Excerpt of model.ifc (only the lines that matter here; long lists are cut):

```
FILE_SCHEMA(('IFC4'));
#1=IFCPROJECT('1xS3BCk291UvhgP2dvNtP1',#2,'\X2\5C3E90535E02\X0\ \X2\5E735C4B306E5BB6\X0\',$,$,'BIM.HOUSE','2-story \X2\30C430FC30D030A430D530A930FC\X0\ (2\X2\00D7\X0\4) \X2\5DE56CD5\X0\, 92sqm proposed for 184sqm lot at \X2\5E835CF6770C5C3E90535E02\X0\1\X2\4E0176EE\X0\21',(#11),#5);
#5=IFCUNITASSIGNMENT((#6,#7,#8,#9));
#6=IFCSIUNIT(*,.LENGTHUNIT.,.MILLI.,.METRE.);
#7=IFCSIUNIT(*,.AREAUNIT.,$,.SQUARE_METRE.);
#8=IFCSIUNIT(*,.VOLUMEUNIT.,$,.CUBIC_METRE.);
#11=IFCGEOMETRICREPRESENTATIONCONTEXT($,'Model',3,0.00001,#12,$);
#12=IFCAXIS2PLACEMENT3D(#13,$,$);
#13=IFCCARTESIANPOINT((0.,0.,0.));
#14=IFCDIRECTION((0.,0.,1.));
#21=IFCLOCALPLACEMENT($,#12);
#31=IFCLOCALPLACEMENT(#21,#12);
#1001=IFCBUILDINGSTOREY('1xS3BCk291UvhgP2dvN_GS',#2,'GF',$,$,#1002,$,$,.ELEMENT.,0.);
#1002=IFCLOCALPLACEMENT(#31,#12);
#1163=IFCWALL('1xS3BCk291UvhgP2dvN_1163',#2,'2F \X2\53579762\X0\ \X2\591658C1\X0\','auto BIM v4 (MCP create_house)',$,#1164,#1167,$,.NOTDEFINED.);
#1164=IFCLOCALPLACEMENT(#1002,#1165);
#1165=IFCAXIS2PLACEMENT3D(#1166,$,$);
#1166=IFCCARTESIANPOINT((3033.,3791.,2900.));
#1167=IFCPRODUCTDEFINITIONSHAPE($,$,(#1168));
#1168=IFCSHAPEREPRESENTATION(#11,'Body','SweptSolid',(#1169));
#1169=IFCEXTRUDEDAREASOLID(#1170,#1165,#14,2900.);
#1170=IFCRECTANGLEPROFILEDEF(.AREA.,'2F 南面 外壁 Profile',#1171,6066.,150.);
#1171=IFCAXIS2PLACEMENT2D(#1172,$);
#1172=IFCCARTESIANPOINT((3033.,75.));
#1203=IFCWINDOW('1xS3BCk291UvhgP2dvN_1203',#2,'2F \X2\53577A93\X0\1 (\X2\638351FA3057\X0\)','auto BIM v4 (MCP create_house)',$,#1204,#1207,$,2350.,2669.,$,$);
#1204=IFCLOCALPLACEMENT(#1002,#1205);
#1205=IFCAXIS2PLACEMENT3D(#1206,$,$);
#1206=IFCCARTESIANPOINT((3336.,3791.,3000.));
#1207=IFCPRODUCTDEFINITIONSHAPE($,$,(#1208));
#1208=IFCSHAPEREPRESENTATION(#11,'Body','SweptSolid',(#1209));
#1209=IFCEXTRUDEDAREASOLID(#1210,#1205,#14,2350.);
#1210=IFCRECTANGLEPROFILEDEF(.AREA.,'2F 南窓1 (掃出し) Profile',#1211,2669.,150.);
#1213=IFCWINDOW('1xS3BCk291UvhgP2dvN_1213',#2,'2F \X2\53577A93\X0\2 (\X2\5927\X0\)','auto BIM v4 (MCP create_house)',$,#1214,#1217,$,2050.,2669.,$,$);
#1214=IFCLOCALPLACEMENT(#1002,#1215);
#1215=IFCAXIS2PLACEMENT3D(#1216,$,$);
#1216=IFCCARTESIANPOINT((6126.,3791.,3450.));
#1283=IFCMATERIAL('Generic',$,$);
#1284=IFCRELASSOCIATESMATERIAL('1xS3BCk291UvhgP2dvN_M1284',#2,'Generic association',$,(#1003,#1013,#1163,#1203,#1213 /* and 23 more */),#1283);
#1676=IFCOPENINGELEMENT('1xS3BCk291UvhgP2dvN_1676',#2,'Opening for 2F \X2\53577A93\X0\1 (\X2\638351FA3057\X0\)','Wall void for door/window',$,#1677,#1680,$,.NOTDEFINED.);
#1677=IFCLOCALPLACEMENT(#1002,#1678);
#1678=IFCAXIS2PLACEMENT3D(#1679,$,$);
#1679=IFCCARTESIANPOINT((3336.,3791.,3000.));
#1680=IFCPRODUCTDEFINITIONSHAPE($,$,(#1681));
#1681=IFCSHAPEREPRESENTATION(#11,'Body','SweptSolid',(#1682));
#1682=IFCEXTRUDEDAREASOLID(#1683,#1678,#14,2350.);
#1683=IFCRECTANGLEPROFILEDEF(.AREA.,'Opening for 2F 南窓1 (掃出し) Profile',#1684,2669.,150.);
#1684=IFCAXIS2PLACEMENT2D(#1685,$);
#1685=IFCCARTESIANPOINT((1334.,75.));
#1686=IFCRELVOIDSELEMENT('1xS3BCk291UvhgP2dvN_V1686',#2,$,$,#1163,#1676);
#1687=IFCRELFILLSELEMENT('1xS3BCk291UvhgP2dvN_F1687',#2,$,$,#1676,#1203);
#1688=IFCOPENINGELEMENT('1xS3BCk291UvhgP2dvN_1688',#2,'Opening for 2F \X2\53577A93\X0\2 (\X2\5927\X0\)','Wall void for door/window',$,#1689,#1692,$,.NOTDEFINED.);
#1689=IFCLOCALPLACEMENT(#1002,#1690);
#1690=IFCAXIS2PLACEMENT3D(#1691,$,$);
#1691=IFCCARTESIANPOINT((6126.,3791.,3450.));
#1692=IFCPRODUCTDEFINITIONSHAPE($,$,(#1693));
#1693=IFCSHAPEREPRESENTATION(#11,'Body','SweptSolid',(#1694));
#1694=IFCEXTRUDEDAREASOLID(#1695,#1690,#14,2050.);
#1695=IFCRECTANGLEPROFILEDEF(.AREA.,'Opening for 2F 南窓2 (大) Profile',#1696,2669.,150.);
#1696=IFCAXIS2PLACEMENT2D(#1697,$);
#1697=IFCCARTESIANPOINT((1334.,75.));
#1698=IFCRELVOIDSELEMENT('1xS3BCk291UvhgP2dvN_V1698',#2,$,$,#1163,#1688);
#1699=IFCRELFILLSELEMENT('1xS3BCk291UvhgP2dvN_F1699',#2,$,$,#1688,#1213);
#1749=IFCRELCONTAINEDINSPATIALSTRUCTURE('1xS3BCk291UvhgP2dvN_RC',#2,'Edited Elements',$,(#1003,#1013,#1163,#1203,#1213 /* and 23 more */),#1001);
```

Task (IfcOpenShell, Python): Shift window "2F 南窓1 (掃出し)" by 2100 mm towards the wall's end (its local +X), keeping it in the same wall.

```python
import ifcopenshell
import ifcopenshell.api.geometry
import ifcopenshell.util.placement
import ifcopenshell.util.unit

model = ifcopenshell.open("model.ifc")
unit_scale = ifcopenshell.util.unit.calculate_unit_scale(model)

window = model.by_guid("1xS3BCk291UvhgP2dvN_1203")
opening = window.FillsVoids[0].RelatingOpeningElement
wall = opening.VoidsElements[0].RelatingBuildingElement

wall_matrix = ifcopenshell.util.placement.get_local_placement(wall.ObjectPlacement)
shift = wall_matrix[:3, 0] * 2.1 / unit_scale
before = ifcopenshell.util.placement.get_local_placement(window.ObjectPlacement)[:3, 3].copy()

# The window is not placed relative to its opening, so move both.
for product in (opening, window):
    matrix = ifcopenshell.util.placement.get_local_placement(product.ObjectPlacement)
    matrix[:3, 3] += shift
    ifcopenshell.api.geometry.edit_object_placement(model, product=product, matrix=matrix, is_si=False)

after = ifcopenshell.util.placement.get_local_placement(window.ObjectPlacement)[:3, 3]
print("window moved by", (after - before).round(3) + 0.0)

model.write("model_updated.ifc")
```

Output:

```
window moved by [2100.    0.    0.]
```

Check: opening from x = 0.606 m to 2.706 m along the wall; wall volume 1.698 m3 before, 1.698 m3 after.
